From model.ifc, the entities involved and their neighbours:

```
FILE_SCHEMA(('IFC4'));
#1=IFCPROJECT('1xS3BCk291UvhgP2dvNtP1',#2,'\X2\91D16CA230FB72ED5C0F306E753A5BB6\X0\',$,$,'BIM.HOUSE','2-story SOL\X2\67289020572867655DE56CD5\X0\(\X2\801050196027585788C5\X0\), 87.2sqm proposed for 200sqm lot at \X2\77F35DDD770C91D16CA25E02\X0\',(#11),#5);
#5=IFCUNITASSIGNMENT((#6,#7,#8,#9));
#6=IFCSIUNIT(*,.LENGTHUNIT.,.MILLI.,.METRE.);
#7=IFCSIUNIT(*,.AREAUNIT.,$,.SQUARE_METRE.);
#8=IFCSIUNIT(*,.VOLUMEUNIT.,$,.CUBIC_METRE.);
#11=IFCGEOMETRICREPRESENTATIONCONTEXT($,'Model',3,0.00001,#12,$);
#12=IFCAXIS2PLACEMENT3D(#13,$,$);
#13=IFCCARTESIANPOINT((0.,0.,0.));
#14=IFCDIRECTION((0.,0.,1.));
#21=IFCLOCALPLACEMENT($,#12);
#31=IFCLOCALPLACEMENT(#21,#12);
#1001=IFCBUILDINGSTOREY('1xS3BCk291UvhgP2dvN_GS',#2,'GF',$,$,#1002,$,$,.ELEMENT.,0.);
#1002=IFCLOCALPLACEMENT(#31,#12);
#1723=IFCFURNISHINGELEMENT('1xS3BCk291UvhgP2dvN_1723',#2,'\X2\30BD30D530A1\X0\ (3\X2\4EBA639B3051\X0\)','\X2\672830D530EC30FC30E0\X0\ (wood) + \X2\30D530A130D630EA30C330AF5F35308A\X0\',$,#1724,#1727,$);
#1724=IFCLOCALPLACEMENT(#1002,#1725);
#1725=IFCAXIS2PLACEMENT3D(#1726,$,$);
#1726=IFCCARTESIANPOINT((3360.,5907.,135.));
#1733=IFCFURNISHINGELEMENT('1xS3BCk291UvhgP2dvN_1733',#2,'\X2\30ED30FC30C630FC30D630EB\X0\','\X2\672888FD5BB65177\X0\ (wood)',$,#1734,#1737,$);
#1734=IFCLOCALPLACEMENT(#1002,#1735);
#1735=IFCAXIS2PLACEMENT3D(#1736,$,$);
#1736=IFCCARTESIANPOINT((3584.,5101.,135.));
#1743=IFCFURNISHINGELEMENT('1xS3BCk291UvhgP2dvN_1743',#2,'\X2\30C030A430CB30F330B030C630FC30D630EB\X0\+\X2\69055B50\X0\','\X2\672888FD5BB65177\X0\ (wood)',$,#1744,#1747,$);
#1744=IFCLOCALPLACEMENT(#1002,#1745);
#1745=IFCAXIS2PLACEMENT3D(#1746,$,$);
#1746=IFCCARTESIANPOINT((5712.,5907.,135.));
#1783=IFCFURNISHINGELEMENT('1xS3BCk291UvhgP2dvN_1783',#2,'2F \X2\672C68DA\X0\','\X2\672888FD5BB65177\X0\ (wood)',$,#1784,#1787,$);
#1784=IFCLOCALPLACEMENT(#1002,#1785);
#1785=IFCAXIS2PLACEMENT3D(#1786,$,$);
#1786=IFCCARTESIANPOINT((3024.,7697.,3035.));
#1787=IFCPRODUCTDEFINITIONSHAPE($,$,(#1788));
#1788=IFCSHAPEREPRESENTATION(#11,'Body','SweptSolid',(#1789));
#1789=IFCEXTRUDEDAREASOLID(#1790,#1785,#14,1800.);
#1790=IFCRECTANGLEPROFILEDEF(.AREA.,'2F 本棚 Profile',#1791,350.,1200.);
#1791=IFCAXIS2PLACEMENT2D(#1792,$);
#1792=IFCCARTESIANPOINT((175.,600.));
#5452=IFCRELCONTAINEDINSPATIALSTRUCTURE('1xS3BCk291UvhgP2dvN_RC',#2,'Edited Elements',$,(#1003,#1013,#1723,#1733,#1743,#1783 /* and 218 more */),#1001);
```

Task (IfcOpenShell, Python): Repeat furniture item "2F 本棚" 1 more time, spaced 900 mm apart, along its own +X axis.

```python
import ifcopenshell
import ifcopenshell.api.geometry
import ifcopenshell.api.root
import ifcopenshell.util.element
import ifcopenshell.util.placement

model = ifcopenshell.open("model.ifc")


def reuse_history(source, copy):
    """copy_class also copies each property set's owner history, people and application; keep the originals."""
    for rel in copy.IsDefinedBy:
        if rel.is_a("IfcRelDefinesByProperties") and (history := rel.RelatingPropertyDefinition.OwnerHistory):
            rel.RelatingPropertyDefinition.OwnerHistory = source.OwnerHistory
            ifcopenshell.util.element.remove_deep2(model, history)


source = model.by_id(1783)
base = ifcopenshell.util.placement.get_local_placement(source.ObjectPlacement)
step = base[:3, 0] * 900.0

for i in range(1, 2):
    copy = ifcopenshell.api.root.copy_class(model, product=source)
    copy.Representation = ifcopenshell.util.element.copy_deep(
        model, source.Representation, exclude=["IfcGeometricRepresentationContext", "IfcRepresentationMap"]
    )
    reuse_history(source, copy)
    matrix = base.copy()
    matrix[:3, 3] += i * step
    print("added at", matrix[:3, 3].round(3) + 0.0)
    ifcopenshell.api.geometry.edit_object_placement(model, product=copy, matrix=matrix, is_si=False)

model.write("model_edited.ifc")
```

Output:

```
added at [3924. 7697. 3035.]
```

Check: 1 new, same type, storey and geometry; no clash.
